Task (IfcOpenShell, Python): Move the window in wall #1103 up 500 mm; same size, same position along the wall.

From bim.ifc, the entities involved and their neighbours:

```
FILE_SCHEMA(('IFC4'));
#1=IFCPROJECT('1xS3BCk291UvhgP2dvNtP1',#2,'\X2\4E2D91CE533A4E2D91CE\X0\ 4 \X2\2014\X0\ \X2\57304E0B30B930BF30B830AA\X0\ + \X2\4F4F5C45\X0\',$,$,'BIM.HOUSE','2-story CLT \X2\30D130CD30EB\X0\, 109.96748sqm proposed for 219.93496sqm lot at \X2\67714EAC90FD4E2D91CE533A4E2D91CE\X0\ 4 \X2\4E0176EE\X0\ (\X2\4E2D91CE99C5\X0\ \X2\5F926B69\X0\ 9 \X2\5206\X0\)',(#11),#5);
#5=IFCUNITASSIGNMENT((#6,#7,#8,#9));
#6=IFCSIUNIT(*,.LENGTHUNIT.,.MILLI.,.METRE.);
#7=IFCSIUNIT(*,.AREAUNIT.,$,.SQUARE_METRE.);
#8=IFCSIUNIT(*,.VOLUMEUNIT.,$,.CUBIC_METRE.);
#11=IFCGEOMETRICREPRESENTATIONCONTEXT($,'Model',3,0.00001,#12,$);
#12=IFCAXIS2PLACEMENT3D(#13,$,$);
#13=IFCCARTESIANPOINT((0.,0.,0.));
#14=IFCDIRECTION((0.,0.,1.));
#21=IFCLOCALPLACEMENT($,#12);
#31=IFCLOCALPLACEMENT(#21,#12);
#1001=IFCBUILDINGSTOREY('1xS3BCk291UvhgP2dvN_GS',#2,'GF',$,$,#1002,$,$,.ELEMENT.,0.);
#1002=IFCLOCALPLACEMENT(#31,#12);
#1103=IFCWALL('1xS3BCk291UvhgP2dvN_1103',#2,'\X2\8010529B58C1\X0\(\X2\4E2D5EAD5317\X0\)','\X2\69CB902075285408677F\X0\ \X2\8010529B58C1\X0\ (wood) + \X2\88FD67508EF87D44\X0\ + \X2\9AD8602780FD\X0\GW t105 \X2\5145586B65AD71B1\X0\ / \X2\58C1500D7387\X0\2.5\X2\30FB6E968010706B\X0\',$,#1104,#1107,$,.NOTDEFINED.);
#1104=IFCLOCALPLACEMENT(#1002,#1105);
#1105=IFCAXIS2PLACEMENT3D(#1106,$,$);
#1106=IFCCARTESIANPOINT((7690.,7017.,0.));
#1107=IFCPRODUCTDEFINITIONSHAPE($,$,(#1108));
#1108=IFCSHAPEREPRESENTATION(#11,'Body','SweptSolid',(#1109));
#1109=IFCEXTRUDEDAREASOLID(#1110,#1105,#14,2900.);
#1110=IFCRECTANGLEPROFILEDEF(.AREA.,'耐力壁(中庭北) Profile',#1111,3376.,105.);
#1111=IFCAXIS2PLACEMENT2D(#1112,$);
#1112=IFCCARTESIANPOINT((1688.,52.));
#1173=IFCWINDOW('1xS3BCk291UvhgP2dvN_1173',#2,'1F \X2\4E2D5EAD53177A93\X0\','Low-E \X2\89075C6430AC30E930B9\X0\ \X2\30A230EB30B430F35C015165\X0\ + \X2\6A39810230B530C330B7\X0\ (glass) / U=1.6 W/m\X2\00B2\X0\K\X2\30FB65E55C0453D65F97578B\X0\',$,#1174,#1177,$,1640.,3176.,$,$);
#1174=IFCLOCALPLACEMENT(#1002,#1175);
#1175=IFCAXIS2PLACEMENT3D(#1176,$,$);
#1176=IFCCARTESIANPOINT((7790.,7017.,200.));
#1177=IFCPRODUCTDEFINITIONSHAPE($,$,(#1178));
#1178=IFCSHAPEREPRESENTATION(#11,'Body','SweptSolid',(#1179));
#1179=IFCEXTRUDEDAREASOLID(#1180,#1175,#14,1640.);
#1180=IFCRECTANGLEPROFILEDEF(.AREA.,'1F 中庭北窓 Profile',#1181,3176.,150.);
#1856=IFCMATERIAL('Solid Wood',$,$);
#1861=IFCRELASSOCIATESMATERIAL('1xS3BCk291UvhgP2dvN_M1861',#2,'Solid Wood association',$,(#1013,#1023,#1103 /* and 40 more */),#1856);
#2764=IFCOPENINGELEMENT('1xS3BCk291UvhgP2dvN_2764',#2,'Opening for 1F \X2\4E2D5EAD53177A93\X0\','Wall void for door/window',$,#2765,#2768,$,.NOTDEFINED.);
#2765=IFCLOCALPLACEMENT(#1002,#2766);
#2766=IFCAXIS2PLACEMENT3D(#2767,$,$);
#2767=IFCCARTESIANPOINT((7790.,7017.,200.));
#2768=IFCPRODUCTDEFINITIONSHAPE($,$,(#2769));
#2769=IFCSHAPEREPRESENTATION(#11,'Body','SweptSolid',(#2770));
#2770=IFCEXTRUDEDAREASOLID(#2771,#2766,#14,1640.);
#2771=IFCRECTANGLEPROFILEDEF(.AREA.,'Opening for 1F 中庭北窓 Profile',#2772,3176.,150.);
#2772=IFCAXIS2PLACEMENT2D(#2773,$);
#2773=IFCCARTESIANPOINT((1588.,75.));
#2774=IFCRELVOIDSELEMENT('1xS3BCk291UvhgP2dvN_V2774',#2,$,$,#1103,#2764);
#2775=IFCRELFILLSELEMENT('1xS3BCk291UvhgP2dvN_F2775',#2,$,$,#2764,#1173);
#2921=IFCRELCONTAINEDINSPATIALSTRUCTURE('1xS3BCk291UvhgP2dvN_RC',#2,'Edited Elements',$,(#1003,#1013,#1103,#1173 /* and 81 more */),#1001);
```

```python
import numpy as np
import ifcopenshell
import ifcopenshell.api.geometry
import ifcopenshell.util.placement
import ifcopenshell.util.unit

model = ifcopenshell.open("bim.ifc")
unit_scale = ifcopenshell.util.unit.calculate_unit_scale(model)

window = model.by_id(1173)
opening = window.FillsVoids[0].RelatingOpeningElement
dz = 500.0

shift = np.array([0.0, 0.0, dz])
# The window is not placed relative to its opening, so move both.
for product in (opening, window):
    matrix = ifcopenshell.util.placement.get_local_placement(product.ObjectPlacement)
    matrix[:3, 3] += shift
    ifcopenshell.api.geometry.edit_object_placement(model, product=product, matrix=matrix, is_si=False)

print(f"moved by {dz * unit_scale:+.3f} m")

model.write("bim-out.ifc")
```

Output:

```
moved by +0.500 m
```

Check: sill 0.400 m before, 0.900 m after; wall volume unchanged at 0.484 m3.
